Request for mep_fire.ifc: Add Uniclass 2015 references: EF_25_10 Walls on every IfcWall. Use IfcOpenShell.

First a look at what the model holds.

```python
import ifcopenshell

model = ifcopenshell.open("mep_fire.ifc")
print(model.schema)
print("classifications:", [c.Name for c in model.by_type("IfcClassification")])
for ifc_class in ("IfcDoor", "IfcRoof", "IfcStair", "IfcWall", "IfcWindow"):
    print(ifc_class, len(model.by_type(ifc_class)))
```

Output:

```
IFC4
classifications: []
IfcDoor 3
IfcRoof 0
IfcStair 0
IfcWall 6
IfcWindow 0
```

```python
import ifcopenshell
import ifcopenshell.api.classification

model = ifcopenshell.open("mep_fire.ifc")

system = ifcopenshell.api.classification.add_classification(model, classification="Uniclass 2015")

codes = {
    "IfcWall": ("EF_25_10", "Walls"),
}
for ifc_class, (code, name) in codes.items():
    products = model.by_type(ifc_class)
    ifcopenshell.api.classification.add_reference(
        model, products=products, classification=system, identification=code, name=name
    )
    print(code, len(products))

model.write("mep_fire_v2.ifc")
```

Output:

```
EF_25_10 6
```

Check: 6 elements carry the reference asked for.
